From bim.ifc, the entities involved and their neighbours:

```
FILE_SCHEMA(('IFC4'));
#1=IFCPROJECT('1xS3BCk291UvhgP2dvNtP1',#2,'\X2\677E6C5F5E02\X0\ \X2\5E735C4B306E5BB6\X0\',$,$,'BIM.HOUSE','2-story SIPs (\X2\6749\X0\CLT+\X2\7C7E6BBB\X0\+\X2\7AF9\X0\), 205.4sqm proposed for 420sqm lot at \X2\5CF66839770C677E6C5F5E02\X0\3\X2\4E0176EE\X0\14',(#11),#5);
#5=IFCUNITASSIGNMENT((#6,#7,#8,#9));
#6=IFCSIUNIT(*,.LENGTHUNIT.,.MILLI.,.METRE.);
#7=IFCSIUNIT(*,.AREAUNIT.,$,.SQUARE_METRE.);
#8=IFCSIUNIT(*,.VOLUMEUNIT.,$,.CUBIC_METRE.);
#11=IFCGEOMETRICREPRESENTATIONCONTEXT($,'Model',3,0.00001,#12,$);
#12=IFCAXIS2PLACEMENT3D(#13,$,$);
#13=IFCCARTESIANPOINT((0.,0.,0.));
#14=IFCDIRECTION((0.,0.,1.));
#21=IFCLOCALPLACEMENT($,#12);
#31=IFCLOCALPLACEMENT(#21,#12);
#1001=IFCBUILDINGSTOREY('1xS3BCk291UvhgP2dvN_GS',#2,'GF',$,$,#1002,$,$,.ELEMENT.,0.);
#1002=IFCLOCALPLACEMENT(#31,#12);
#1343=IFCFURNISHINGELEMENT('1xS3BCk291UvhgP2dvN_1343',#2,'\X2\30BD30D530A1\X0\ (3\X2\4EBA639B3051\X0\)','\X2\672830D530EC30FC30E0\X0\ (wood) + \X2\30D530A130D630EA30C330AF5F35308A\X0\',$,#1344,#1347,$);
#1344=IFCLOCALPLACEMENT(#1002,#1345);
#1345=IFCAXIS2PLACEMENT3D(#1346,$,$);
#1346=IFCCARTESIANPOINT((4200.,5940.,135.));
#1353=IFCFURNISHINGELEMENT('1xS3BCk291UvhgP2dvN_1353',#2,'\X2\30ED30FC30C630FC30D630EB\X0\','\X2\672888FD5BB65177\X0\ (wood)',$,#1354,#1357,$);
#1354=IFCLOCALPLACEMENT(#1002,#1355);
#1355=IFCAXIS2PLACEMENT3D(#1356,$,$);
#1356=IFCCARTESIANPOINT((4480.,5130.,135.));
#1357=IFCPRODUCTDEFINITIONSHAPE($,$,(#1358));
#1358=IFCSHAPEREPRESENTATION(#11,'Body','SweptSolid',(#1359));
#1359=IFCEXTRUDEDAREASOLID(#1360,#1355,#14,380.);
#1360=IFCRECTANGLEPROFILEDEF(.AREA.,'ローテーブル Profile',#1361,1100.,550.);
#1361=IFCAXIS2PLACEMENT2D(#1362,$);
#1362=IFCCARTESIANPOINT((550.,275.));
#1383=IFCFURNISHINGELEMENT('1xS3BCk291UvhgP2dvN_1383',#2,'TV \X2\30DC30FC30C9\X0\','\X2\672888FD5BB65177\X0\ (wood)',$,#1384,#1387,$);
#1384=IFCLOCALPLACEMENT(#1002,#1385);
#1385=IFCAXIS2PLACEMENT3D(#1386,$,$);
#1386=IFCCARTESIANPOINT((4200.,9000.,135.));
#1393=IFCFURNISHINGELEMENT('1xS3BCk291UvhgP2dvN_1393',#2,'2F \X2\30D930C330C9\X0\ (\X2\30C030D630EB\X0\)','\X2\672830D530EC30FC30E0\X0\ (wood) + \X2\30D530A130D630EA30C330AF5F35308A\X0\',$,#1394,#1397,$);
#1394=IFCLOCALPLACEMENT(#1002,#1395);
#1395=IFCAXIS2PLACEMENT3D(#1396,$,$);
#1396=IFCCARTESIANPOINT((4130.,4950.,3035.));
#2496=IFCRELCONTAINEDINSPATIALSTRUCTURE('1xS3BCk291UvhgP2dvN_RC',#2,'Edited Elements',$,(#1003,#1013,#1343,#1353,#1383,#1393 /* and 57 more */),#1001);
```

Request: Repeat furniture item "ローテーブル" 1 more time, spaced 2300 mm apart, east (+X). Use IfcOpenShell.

```python
import numpy as np
import ifcopenshell
import ifcopenshell.api.geometry
import ifcopenshell.api.root
import ifcopenshell.util.element
import ifcopenshell.util.placement

model = ifcopenshell.open("bim.ifc")


def reuse_history(source, copy):
    """copy_class also copies each property set's owner history, people and application; keep the originals."""
    for rel in copy.IsDefinedBy:
        if rel.is_a("IfcRelDefinesByProperties") and (history := rel.RelatingPropertyDefinition.OwnerHistory):
            rel.RelatingPropertyDefinition.OwnerHistory = source.OwnerHistory
            ifcopenshell.util.element.remove_deep2(model, history)


source = model.by_guid("1xS3BCk291UvhgP2dvN_1353")
base = ifcopenshell.util.placement.get_local_placement(source.ObjectPlacement)
step = np.array([1.0, 0.0, 0.0]) * 2300.0

for i in range(1, 2):
    copy = ifcopenshell.api.root.copy_class(model, product=source)
    copy.Representation = ifcopenshell.util.element.copy_deep(
        model, source.Representation, exclude=["IfcGeometricRepresentationContext", "IfcRepresentationMap"]
    )
    reuse_history(source, copy)
    matrix = base.copy()
    matrix[:3, 3] += i * step
    print("added at", matrix[:3, 3].round(3) + 0.0)
    ifcopenshell.api.geometry.edit_object_placement(model, product=copy, matrix=matrix, is_si=False)

model.write("bim_edited.ifc")
```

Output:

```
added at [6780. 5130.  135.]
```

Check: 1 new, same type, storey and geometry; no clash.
